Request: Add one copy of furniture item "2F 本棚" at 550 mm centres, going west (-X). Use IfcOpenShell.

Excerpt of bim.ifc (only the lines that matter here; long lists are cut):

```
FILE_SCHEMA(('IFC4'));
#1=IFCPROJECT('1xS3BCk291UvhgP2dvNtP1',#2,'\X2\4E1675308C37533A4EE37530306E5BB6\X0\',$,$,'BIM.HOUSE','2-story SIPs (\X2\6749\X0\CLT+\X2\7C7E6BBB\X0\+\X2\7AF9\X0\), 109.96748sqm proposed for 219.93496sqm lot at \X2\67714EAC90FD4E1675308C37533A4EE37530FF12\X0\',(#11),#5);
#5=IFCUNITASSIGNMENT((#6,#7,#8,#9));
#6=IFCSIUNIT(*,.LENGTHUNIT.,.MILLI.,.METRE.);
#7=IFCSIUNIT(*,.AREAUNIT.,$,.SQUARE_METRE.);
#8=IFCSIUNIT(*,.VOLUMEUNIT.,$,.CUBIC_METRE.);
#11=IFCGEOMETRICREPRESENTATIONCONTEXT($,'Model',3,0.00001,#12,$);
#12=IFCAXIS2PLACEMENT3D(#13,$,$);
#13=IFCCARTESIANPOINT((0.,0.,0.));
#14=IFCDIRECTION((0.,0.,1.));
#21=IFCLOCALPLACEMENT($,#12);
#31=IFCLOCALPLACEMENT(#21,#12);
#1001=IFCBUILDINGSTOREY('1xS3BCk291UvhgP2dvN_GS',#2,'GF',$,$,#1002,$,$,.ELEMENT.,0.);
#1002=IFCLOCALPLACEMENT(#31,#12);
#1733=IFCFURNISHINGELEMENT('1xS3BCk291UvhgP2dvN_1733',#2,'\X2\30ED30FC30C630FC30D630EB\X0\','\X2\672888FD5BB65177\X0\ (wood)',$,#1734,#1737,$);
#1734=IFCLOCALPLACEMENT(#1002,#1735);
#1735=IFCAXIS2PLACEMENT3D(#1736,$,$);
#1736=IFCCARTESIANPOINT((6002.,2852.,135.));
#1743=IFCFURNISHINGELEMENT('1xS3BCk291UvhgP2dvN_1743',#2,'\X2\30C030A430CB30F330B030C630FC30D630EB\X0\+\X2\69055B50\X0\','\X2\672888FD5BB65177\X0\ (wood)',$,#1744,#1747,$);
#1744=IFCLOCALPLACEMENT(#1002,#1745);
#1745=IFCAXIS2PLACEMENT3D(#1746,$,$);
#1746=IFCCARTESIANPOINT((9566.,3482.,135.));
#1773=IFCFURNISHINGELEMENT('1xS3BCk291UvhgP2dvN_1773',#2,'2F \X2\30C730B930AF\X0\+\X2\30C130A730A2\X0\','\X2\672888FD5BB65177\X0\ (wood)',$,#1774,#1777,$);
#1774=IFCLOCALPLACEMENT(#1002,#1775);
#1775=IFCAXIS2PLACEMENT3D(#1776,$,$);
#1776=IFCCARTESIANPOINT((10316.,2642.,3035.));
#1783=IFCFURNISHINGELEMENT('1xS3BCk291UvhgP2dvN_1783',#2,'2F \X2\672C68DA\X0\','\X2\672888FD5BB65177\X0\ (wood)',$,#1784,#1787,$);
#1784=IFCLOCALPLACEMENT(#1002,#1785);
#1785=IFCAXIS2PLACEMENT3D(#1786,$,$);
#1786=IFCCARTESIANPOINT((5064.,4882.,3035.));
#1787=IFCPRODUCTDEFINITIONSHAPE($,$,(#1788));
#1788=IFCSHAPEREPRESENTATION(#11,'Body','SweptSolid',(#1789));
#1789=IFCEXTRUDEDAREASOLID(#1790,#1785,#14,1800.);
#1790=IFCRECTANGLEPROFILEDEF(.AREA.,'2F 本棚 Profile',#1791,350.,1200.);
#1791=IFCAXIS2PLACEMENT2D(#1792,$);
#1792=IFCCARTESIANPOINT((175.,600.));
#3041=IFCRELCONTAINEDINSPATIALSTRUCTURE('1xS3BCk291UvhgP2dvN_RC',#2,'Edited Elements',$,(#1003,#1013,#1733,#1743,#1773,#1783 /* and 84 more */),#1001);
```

```python
import numpy as np
import ifcopenshell
import ifcopenshell.api.geometry
import ifcopenshell.api.root
import ifcopenshell.util.element
import ifcopenshell.util.placement
import ifcopenshell.util.unit

model = ifcopenshell.open("bim.ifc")
unit_scale = ifcopenshell.util.unit.calculate_unit_scale(model)


def reuse_history(source, copy):
    """copy_class also copies each property set's owner history, people and application; keep the originals."""
    for rel in copy.IsDefinedBy:
        if rel.is_a("IfcRelDefinesByProperties") and (history := rel.RelatingPropertyDefinition.OwnerHistory):
            rel.RelatingPropertyDefinition.OwnerHistory = source.OwnerHistory
            ifcopenshell.util.element.remove_deep2(model, history)


source = model.by_guid("1xS3BCk291UvhgP2dvN_1783")
base = ifcopenshell.util.placement.get_local_placement(source.ObjectPlacement)
step = np.array([-1.0, 0.0, 0.0]) * 0.55 / unit_scale

for i in range(1, 2):
    copy = ifcopenshell.api.root.copy_class(model, product=source)
    copy.Representation = ifcopenshell.util.element.copy_deep(
        model, source.Representation, exclude=["IfcGeometricRepresentationContext", "IfcRepresentationMap"]
    )
    reuse_history(source, copy)
    matrix = base.copy()
    matrix[:3, 3] += i * step
    print("added at", matrix[:3, 3].round(3) + 0.0)
    ifcopenshell.api.geometry.edit_object_placement(model, product=copy, matrix=matrix, is_si=False)

model.write("bim_edited.ifc")
```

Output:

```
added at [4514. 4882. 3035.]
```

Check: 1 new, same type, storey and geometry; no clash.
